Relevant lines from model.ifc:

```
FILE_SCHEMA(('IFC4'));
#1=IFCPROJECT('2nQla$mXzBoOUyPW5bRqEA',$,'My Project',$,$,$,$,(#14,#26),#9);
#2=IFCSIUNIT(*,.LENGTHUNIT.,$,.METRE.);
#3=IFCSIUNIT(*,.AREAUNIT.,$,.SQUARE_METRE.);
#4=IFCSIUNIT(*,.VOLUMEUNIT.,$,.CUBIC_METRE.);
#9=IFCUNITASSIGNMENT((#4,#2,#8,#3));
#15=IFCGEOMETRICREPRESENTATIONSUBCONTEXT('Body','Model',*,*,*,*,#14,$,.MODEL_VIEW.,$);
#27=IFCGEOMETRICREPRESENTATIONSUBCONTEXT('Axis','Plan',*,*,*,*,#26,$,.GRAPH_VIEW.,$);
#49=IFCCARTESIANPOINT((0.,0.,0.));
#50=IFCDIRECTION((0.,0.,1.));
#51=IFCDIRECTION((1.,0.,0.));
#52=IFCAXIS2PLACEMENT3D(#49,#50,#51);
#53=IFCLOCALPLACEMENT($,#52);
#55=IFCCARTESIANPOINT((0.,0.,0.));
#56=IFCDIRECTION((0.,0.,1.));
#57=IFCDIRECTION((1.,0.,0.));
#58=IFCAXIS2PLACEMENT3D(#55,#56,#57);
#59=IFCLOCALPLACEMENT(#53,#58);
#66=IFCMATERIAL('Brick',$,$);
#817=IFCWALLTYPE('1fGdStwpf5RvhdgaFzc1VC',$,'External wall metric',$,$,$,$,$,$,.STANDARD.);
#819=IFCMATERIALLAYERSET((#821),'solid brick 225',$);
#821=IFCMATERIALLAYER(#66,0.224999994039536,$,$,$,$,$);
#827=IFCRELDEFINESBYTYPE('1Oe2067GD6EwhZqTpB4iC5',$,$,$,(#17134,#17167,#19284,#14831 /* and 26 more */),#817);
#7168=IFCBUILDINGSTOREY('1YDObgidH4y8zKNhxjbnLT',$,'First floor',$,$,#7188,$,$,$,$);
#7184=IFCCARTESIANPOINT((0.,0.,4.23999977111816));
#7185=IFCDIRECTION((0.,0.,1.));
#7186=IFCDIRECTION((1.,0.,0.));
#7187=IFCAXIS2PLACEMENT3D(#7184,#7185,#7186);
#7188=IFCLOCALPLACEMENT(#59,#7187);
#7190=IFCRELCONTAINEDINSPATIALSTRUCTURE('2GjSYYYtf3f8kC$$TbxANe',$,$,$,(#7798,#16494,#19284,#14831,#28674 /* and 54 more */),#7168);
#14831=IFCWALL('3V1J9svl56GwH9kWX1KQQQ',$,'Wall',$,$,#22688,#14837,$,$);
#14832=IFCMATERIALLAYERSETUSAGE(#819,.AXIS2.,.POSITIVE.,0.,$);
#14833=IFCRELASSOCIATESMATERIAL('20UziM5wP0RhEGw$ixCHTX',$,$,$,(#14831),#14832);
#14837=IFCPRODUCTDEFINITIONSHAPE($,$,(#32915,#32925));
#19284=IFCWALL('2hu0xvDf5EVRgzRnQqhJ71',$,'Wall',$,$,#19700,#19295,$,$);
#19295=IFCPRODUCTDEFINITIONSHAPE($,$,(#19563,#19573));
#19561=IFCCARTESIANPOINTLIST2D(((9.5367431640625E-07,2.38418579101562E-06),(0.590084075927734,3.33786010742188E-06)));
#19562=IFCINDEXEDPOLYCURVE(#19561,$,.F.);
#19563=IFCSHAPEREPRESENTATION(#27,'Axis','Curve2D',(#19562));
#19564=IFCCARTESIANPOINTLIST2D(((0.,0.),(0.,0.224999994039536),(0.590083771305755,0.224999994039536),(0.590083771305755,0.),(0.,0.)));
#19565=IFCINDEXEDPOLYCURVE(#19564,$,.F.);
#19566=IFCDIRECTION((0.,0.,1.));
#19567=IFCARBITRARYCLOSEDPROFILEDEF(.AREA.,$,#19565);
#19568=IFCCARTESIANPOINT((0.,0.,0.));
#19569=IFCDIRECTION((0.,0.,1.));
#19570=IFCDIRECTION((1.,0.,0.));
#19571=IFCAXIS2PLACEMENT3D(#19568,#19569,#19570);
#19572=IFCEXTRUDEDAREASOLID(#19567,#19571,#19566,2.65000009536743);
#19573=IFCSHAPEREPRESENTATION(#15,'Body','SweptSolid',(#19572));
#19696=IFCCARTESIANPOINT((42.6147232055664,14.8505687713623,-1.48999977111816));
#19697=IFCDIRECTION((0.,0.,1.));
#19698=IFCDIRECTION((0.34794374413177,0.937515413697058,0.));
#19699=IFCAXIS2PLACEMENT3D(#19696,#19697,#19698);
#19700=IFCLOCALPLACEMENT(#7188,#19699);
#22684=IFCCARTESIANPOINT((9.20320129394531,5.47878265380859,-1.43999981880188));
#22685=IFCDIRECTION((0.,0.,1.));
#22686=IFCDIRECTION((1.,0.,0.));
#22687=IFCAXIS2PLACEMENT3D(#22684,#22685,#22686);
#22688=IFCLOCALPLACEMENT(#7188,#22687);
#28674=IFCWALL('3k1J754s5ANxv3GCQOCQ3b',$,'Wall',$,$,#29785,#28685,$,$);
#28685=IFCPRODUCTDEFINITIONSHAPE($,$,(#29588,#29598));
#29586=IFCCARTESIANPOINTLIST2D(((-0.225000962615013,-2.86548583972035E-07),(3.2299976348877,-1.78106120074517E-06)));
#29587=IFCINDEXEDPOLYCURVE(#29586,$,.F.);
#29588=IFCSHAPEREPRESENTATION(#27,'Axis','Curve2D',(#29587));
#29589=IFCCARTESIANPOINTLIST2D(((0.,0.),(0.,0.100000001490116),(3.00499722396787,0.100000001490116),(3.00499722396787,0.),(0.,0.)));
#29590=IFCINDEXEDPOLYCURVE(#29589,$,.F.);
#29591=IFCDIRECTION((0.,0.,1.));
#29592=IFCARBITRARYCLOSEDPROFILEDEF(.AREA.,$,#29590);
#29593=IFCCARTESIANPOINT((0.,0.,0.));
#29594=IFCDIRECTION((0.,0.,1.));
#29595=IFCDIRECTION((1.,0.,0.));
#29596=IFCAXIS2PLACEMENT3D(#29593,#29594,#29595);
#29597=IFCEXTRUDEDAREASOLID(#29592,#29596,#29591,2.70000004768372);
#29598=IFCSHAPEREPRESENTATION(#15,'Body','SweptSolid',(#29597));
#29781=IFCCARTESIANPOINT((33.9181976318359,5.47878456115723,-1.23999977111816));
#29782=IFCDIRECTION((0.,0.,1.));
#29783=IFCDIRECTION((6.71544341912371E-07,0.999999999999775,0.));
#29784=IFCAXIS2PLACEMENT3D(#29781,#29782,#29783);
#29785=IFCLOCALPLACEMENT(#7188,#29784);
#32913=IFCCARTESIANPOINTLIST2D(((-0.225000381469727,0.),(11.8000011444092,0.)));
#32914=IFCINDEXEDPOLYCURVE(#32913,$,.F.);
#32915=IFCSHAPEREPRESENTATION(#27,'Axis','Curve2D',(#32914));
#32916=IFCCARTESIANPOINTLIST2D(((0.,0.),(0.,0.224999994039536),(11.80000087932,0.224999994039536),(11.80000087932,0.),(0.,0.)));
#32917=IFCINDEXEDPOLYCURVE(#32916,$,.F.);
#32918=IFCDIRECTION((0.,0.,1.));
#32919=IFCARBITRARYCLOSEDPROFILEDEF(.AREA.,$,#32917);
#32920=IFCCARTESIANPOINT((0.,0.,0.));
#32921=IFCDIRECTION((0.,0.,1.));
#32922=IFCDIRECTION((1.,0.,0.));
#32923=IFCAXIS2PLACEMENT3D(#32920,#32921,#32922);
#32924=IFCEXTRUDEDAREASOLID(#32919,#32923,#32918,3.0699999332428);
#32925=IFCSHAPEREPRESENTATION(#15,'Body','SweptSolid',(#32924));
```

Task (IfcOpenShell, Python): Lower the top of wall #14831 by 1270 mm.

```python
import ifcopenshell
import ifcopenshell.geom
import ifcopenshell.util.representation
import ifcopenshell.util.shape
import ifcopenshell.util.unit

model = ifcopenshell.open("model.ifc")
unit_scale = ifcopenshell.util.unit.calculate_unit_scale(model)
settings = ifcopenshell.geom.settings()


def volume(element):
    """Net volume in cubic metres, openings subtracted."""
    shape = ifcopenshell.geom.create_shape(settings, element)
    return ifcopenshell.util.shape.get_volume(shape.geometry)


wall = model.by_id(14831)
before = volume(wall)

body = ifcopenshell.util.representation.get_representation(wall, "Model", "Body")
solid = body.Items[0]
old_height = solid.Depth
solid.Depth -= 1.27 / unit_scale
after = volume(wall)

print(f"height {old_height:g} -> {solid.Depth:g}, volume {before:.3f} -> {after:.3f} m3")

model.write("model_v2.ifc")
```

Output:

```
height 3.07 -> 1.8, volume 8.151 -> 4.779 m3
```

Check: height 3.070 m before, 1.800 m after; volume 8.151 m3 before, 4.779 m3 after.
